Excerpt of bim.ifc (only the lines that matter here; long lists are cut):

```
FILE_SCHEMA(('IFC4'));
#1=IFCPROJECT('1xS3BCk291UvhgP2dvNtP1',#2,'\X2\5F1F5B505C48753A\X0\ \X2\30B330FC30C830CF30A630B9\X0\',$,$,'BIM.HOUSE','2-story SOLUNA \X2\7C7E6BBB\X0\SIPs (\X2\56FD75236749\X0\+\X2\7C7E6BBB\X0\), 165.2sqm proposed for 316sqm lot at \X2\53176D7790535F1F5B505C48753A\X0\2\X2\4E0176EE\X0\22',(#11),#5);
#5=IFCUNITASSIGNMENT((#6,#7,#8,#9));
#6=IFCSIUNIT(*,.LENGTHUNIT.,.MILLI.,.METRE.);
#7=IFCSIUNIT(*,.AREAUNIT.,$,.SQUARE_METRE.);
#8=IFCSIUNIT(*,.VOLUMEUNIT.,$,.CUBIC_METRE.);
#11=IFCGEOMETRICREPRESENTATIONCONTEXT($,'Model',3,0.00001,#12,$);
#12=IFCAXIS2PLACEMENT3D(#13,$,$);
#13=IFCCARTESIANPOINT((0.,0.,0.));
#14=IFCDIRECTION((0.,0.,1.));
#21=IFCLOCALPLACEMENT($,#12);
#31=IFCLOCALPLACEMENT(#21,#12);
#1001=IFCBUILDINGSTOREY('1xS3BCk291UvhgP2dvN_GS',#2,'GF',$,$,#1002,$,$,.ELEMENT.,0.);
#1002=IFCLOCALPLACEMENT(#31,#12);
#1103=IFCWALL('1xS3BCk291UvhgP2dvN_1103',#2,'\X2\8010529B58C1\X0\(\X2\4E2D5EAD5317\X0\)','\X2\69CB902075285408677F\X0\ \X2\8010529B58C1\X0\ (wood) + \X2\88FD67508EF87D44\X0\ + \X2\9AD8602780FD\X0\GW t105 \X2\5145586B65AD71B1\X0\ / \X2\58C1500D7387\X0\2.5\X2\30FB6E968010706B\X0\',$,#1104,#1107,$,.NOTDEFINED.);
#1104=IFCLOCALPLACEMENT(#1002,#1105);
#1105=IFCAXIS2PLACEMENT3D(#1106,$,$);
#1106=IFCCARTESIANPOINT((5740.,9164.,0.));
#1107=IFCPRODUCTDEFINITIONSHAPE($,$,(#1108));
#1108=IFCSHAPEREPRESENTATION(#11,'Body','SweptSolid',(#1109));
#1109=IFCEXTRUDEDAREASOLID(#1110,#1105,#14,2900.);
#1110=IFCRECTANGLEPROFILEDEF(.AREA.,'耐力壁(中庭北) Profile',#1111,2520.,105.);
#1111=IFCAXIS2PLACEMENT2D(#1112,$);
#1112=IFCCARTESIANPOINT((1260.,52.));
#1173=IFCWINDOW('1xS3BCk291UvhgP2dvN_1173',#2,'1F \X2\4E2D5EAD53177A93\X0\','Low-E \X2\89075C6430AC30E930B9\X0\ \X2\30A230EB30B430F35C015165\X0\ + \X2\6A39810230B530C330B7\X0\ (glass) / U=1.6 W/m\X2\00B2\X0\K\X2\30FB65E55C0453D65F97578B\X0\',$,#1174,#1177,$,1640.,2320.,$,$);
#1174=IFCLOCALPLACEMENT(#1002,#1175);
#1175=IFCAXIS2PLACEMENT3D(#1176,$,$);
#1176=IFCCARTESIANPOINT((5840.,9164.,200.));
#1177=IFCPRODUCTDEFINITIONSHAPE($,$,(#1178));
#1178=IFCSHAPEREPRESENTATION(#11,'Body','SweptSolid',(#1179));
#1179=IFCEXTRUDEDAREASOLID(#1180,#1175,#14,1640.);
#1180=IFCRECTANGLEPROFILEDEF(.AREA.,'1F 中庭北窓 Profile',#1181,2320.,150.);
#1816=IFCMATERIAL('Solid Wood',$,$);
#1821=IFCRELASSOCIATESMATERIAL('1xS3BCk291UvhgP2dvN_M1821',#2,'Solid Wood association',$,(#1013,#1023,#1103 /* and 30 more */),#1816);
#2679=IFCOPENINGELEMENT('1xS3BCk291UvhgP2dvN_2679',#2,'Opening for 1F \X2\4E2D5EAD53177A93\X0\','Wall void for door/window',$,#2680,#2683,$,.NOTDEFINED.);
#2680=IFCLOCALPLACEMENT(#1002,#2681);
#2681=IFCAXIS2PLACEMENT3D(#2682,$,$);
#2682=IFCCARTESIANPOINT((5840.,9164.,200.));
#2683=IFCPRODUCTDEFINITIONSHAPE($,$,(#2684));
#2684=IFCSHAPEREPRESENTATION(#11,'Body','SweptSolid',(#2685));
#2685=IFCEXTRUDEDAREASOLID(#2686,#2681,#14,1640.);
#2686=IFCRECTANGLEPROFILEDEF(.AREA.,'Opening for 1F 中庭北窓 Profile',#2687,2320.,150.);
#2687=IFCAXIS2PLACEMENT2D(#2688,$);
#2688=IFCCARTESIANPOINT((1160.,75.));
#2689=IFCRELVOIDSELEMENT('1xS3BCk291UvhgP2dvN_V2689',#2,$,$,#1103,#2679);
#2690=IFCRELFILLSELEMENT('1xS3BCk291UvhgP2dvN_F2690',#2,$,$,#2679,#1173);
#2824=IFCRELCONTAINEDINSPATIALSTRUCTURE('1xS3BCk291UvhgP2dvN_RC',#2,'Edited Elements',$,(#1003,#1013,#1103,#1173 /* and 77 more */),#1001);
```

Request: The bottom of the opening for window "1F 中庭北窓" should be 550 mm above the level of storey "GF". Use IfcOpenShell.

```python
import numpy as np
import ifcopenshell
import ifcopenshell.api.geometry
import ifcopenshell.geom
import ifcopenshell.util.element
import ifcopenshell.util.placement
import ifcopenshell.util.shape
import ifcopenshell.util.unit

model = ifcopenshell.open("bim.ifc")
unit_scale = ifcopenshell.util.unit.calculate_unit_scale(model)

window = model.by_guid("1xS3BCk291UvhgP2dvN_1173")
opening = window.FillsVoids[0].RelatingOpeningElement
storey = ifcopenshell.util.element.get_container(window, ifc_class="IfcBuildingStorey")
level = ifcopenshell.util.placement.get_local_placement(storey.ObjectPlacement)[2, 3]

# The opening's origin need not be at the sill, so measure its lowest point.
shape = ifcopenshell.geom.create_shape(ifcopenshell.geom.settings(), opening)
bottom = ifcopenshell.util.shape.get_shape_bottom_elevation(shape, shape.geometry) / unit_scale
dz = level + 550.0 - bottom

shift = np.array([0.0, 0.0, dz])
# The window is not placed relative to its opening, so move both.
for product in (opening, window):
    matrix = ifcopenshell.util.placement.get_local_placement(product.ObjectPlacement)
    matrix[:3, 3] += shift
    ifcopenshell.api.geometry.edit_object_placement(model, product=product, matrix=matrix, is_si=False)

print(f"moved by {dz * unit_scale:+.3f} m")

model.write("bim_updated.ifc")
```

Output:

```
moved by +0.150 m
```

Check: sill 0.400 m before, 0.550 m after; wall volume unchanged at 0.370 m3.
